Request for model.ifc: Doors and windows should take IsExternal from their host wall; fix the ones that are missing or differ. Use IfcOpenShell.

First a look at what the model holds.

```python
import ifcopenshell
import ifcopenshell.util.element

model = ifcopenshell.open("model.ifc")
print(model.schema)
seen = {}
for e in model.by_type("IfcDoor") + model.by_type("IfcWindow"):
    if not e.FillsVoids:
        continue
    host = e.FillsVoids[0].RelatingOpeningElement.VoidsElements[0].RelatingBuildingElement
    own = ifcopenshell.util.element.get_pset(e, f"Pset_{e.is_a()[3:].removesuffix('StandardCase')}Common", "IsExternal")
    wall = ifcopenshell.util.element.get_pset(host, "Pset_WallCommon", "IsExternal")
    seen[e.is_a(), own, wall] = seen.get((e.is_a(), own, wall), 0) + 1
for (cls, own, wall), count in sorted(seen.items(), key=str):
    print(count, cls, "IsExternal:", own, "| host wall:", wall)
```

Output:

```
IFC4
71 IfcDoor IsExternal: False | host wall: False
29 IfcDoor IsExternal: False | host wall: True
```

```python
import ifcopenshell
import ifcopenshell.api.pset
import ifcopenshell.util.element

model = ifcopenshell.open("model.ifc")

count = 0
for ifc_class, pset_name in (("IfcDoor", "Pset_DoorCommon"), ("IfcWindow", "Pset_WindowCommon")):
    for e in model.by_type(ifc_class):
        if not e.FillsVoids:
            continue
        host = e.FillsVoids[0].RelatingOpeningElement.VoidsElements[0].RelatingBuildingElement
        external = ifcopenshell.util.element.get_pset(host, "Pset_WallCommon", "IsExternal")
        if external is None or ifcopenshell.util.element.get_pset(e, pset_name, "IsExternal") == external:
            continue
        pset = ifcopenshell.api.pset.add_pset(model, product=e, name=pset_name)
        ifcopenshell.api.pset.edit_pset(model, pset=pset, properties={"IsExternal": external})
        count += 1

print(count, "updated")

model.write("model_rev.ifc")
```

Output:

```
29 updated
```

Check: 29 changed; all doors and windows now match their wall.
